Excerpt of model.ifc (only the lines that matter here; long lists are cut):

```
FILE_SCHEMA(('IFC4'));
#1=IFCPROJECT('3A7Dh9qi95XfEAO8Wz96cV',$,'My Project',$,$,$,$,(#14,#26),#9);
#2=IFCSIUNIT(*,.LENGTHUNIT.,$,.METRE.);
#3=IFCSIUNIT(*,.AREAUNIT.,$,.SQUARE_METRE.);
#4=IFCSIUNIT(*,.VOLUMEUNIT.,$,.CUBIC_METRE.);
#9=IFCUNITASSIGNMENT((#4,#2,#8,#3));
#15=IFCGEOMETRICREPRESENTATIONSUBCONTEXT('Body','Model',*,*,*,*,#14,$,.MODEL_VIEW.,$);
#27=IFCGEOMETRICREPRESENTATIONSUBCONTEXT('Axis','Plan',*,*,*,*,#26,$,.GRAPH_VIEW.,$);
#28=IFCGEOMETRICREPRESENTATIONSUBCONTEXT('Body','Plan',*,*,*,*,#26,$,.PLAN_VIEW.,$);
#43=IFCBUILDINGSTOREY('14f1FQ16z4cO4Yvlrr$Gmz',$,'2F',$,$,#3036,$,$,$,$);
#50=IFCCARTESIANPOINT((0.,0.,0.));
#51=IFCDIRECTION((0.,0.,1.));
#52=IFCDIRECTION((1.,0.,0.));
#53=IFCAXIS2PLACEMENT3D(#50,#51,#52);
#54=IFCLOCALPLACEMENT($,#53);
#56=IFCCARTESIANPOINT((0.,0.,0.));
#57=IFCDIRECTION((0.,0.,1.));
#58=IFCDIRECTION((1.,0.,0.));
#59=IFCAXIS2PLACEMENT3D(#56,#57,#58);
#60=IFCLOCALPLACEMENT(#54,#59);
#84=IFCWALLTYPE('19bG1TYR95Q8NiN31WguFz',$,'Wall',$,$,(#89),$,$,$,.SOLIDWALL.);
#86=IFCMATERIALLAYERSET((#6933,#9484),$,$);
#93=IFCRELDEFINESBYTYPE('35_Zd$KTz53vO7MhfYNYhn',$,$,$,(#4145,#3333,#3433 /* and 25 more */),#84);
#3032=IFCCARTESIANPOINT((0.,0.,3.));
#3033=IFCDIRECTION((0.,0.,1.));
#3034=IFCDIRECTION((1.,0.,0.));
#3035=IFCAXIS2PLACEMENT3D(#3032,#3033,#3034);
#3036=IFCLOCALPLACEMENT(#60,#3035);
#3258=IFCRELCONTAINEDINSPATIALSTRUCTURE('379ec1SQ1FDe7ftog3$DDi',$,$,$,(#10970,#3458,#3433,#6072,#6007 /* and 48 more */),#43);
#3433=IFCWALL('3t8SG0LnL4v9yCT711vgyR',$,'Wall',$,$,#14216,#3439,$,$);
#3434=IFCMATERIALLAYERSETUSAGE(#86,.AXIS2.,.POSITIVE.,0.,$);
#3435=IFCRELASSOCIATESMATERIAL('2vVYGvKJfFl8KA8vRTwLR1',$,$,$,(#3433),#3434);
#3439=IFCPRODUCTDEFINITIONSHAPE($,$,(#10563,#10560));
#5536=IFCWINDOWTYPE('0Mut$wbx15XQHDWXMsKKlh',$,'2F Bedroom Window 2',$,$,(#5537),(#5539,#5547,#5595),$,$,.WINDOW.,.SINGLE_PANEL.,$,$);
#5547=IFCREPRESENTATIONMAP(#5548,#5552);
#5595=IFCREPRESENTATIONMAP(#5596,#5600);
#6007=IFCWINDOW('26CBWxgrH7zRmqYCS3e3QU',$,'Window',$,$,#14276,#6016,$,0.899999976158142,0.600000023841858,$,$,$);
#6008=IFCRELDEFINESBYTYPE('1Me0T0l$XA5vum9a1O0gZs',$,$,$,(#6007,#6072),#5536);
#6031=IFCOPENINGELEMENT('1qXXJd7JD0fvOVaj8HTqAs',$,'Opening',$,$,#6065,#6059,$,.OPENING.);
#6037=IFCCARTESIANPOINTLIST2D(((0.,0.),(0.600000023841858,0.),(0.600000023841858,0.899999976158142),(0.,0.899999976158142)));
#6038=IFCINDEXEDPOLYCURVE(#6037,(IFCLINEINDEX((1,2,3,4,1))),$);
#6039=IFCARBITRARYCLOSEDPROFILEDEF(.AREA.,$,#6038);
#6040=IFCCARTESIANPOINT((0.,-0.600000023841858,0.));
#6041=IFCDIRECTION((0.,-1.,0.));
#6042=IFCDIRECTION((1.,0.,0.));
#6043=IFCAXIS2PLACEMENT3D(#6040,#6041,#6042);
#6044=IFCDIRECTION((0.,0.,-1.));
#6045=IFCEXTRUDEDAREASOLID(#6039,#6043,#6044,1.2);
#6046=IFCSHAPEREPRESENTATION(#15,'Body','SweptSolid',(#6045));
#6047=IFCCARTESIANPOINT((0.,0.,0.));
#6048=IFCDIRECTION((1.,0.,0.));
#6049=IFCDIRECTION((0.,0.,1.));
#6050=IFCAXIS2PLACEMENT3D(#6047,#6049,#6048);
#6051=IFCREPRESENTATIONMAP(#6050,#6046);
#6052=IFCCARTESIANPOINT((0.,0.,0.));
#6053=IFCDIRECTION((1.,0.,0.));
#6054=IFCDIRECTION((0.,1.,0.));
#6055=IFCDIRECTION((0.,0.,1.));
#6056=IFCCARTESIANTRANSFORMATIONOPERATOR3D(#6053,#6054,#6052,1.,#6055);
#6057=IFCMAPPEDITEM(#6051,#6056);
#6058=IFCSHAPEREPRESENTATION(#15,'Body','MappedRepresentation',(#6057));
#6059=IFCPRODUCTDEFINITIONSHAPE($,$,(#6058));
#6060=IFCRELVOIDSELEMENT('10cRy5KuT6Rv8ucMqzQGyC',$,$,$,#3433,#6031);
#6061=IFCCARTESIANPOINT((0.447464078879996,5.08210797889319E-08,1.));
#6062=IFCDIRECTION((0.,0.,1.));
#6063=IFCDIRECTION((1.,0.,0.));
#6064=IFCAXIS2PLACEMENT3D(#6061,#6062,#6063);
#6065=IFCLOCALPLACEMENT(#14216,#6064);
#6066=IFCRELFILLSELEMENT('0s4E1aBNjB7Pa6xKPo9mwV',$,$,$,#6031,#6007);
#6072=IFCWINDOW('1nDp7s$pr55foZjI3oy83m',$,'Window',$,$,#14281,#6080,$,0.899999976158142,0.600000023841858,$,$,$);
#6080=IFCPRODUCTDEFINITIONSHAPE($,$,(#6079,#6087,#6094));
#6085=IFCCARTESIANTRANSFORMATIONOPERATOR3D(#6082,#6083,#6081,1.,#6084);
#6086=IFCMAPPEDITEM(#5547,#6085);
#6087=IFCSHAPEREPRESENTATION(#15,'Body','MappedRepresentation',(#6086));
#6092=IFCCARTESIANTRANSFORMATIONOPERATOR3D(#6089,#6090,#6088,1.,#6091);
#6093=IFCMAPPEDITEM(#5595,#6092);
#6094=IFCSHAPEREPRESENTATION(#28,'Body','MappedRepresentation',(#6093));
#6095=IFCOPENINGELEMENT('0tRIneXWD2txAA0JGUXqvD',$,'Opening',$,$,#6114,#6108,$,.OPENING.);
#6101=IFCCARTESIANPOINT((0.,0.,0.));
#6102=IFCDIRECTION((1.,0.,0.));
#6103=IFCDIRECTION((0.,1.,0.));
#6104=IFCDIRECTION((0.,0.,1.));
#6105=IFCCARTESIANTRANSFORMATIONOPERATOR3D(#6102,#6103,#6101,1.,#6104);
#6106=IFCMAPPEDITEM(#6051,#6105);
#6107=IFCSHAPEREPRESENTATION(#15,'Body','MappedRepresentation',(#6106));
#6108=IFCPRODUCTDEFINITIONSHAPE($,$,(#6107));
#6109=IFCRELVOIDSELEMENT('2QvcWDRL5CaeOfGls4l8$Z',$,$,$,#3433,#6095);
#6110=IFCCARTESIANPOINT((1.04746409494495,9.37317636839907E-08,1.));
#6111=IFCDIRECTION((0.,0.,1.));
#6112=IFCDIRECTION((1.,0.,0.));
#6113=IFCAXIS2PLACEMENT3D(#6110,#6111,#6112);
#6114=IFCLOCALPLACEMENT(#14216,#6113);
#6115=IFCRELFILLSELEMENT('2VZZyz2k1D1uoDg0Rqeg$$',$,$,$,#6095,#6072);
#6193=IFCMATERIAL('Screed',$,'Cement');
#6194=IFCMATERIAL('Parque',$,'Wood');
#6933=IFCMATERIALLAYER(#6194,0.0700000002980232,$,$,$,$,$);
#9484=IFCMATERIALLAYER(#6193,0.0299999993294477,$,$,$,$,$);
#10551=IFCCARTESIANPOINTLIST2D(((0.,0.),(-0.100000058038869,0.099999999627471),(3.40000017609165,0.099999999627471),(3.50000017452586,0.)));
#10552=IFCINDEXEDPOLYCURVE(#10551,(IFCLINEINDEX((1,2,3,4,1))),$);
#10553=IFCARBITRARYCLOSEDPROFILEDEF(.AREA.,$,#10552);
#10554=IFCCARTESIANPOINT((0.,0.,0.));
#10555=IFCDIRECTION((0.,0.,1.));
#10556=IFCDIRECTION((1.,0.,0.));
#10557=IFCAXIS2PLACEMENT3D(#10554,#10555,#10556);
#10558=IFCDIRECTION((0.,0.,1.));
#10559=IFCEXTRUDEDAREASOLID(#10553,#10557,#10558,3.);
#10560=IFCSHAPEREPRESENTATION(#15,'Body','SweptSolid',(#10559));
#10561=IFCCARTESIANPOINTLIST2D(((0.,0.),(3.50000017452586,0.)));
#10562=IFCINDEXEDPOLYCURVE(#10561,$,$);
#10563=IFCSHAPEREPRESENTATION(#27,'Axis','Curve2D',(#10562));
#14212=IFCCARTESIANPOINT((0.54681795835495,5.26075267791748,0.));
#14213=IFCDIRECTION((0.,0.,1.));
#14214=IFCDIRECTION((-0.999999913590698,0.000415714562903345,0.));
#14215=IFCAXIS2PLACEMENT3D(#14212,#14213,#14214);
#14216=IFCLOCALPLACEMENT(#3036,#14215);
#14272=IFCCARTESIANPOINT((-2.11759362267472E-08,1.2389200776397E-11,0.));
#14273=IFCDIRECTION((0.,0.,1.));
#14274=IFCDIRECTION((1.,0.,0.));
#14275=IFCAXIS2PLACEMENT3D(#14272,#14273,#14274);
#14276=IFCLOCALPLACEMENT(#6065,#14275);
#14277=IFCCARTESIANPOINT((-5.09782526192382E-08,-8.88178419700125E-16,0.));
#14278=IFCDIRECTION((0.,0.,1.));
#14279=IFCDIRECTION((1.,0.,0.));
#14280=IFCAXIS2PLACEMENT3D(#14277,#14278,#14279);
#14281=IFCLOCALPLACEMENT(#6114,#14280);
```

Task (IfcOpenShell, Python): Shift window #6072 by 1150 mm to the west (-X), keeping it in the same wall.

```python
import ifcopenshell
import ifcopenshell.api.geometry
import ifcopenshell.util.placement
import ifcopenshell.util.unit

model = ifcopenshell.open("model.ifc")
unit_scale = ifcopenshell.util.unit.calculate_unit_scale(model)

window = model.by_guid("1nDp7s$pr55foZjI3oy83m")
opening = window.FillsVoids[0].RelatingOpeningElement
wall = opening.VoidsElements[0].RelatingBuildingElement

wall_matrix = ifcopenshell.util.placement.get_local_placement(wall.ObjectPlacement)
shift = wall_matrix[:3, 0] * 1.15 / unit_scale
before = ifcopenshell.util.placement.get_local_placement(window.ObjectPlacement)[:3, 3].copy()

# The window is placed relative to its opening, so it follows when the opening moves.
matrix = ifcopenshell.util.placement.get_local_placement(opening.ObjectPlacement)
matrix[:3, 3] += shift
ifcopenshell.api.geometry.edit_object_placement(
    model, product=opening, matrix=matrix, is_si=False, should_transform_children=True
)

after = ifcopenshell.util.placement.get_local_placement(window.ObjectPlacement)[:3, 3]
print("window moved by", (after - before).round(3) + 0.0)

model.write("model-out.ifc")
```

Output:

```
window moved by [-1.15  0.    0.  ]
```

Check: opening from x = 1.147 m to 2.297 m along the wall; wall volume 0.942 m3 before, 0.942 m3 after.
